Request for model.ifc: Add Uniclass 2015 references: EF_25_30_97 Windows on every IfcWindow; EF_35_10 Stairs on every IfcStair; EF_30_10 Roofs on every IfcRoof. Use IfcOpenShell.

First a look at what the model holds.

```python
import ifcopenshell

model = ifcopenshell.open("model.ifc")
print(model.schema)
print("classifications:", [c.Name for c in model.by_type("IfcClassification")])
for ifc_class in ("IfcDoor", "IfcRoof", "IfcStair", "IfcWall", "IfcWindow"):
    print(ifc_class, len(model.by_type(ifc_class)))
```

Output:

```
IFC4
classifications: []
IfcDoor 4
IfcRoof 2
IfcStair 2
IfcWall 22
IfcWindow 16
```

```python
import ifcopenshell
import ifcopenshell.api.classification

model = ifcopenshell.open("model.ifc")

system = ifcopenshell.api.classification.add_classification(model, classification="Uniclass 2015")

codes = {
    "IfcWindow": ("EF_25_30_97", "Windows"),
    "IfcStair": ("EF_35_10", "Stairs"),
    "IfcRoof": ("EF_30_10", "Roofs"),
}
for ifc_class, (code, name) in codes.items():
    products = model.by_type(ifc_class)
    ifcopenshell.api.classification.add_reference(
        model, products=products, classification=system, identification=code, name=name
    )
    print(code, len(products))

model.write("model-out.ifc")
```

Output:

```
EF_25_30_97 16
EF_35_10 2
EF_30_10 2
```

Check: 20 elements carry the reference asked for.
